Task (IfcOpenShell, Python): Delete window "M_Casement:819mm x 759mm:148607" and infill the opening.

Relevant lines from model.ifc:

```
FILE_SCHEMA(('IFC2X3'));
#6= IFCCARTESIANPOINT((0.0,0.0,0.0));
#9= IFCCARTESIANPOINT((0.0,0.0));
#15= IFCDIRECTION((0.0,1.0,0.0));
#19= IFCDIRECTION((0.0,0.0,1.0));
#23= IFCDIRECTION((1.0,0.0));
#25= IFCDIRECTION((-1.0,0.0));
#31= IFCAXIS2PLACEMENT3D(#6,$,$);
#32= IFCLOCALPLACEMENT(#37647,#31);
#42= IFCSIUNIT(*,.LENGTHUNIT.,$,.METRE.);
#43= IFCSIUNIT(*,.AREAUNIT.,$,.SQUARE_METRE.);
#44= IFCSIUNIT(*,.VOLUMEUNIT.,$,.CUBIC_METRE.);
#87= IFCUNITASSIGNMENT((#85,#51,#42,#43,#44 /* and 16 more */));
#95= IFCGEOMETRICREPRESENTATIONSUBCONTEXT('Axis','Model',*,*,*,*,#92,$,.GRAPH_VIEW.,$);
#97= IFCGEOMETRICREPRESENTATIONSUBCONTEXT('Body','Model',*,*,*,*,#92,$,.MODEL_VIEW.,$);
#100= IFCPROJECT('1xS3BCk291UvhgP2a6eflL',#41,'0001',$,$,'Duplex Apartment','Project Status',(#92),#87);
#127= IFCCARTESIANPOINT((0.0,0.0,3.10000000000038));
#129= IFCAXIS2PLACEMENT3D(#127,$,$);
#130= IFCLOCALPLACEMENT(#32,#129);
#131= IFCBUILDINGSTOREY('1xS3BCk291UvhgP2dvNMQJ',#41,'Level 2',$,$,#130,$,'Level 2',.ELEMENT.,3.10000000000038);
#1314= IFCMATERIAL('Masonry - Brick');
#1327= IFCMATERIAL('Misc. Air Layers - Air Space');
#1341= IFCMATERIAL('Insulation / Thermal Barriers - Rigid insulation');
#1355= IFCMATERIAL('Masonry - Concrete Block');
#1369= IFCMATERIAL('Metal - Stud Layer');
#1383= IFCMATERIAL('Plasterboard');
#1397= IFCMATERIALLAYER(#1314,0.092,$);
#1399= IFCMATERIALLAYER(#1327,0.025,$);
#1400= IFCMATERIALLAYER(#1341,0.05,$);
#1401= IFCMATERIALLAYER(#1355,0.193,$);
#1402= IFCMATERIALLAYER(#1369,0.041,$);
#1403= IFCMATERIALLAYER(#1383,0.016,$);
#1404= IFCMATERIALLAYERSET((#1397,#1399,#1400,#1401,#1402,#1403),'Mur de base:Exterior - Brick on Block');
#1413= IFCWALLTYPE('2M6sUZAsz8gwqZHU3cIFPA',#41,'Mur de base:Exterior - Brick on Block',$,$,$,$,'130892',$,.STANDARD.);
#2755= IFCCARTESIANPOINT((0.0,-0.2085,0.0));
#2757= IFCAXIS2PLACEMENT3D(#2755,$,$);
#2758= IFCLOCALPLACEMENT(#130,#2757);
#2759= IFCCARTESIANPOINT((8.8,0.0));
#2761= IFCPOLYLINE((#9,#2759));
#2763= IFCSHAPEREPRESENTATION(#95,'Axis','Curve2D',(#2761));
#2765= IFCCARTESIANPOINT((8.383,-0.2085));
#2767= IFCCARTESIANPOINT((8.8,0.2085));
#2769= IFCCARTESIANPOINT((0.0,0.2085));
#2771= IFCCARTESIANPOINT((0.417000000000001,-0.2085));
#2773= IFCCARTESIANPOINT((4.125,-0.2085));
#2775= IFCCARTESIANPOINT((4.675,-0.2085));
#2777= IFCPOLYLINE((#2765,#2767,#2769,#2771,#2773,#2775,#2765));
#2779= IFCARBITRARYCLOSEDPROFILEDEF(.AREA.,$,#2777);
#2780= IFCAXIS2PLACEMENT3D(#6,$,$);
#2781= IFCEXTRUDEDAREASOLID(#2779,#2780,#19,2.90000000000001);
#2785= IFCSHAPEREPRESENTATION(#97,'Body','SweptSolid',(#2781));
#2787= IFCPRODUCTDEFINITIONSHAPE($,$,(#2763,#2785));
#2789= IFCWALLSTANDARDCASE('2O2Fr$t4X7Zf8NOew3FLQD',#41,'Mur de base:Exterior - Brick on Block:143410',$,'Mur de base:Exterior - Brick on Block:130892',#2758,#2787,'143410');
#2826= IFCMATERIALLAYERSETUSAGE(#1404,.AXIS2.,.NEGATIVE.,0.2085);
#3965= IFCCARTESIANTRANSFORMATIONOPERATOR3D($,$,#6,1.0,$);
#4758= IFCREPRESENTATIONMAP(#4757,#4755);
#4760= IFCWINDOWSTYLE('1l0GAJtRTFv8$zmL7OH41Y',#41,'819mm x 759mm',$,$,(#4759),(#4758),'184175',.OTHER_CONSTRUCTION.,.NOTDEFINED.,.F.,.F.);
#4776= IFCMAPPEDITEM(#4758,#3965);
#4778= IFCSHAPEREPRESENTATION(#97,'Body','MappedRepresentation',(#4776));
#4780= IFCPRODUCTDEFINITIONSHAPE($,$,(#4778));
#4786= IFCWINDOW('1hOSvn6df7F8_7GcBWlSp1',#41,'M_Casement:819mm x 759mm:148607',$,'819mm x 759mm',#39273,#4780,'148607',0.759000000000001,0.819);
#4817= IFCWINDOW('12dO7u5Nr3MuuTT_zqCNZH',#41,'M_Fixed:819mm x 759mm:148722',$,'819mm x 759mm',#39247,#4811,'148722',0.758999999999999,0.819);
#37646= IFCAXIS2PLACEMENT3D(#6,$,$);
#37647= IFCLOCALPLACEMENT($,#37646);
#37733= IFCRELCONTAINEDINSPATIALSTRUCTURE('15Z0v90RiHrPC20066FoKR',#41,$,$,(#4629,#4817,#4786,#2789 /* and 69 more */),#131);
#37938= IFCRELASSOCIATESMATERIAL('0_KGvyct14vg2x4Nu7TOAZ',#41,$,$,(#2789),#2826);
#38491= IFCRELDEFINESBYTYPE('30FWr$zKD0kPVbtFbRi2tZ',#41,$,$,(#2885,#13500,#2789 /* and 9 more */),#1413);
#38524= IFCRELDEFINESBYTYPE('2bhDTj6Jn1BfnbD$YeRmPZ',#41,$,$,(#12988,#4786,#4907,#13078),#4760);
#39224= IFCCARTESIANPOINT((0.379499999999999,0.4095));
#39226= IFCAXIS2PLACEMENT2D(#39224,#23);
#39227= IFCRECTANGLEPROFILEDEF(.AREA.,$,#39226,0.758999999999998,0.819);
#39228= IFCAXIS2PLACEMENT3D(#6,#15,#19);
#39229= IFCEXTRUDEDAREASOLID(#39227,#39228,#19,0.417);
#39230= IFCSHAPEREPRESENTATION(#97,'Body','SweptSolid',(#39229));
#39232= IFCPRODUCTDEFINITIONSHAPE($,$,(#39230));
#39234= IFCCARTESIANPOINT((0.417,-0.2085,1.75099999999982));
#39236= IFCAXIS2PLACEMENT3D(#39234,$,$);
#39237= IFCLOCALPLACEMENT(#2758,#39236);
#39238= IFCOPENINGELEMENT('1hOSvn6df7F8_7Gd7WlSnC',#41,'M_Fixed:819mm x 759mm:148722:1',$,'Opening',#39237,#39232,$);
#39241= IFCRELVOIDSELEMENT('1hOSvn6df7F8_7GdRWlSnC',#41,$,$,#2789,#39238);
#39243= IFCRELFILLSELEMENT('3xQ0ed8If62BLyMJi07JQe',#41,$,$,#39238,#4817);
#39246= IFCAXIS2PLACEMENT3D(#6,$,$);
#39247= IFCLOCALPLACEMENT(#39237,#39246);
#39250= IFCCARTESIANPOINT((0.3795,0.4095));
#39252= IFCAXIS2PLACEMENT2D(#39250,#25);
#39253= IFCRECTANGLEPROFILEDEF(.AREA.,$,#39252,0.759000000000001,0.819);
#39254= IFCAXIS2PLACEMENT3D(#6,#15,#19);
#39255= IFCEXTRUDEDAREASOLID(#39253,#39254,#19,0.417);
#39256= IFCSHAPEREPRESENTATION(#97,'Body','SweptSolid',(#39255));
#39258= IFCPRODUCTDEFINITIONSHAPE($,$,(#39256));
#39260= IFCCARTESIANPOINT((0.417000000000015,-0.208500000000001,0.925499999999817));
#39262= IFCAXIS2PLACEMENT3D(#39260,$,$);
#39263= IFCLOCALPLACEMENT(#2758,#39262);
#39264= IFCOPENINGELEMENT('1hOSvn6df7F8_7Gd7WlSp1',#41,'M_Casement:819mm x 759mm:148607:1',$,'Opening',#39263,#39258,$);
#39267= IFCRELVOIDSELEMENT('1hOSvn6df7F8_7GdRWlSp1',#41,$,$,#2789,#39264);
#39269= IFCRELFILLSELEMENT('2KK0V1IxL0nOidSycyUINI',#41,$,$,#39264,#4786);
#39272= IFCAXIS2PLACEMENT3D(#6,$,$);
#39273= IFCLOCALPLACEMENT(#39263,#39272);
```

```python
import ifcopenshell
import ifcopenshell.api.feature
import ifcopenshell.api.root
import ifcopenshell.geom
import ifcopenshell.util.shape

model = ifcopenshell.open("model.ifc")
settings = ifcopenshell.geom.settings()


def volume(element):
    """Net volume in cubic metres, openings subtracted."""
    shape = ifcopenshell.geom.create_shape(settings, element)
    return ifcopenshell.util.shape.get_volume(shape.geometry)


window = model.by_id(4786)
opening = window.FillsVoids[0].RelatingOpeningElement
wall = opening.VoidsElements[0].RelatingBuildingElement
before = volume(wall)

ifcopenshell.api.root.remove_product(model, product=window)
ifcopenshell.api.feature.remove_feature(model, feature=opening)

after = volume(wall)

print(f"wall volume {before:.3f} -> {after:.3f} m3")

model.write("model_v2.ifc")
```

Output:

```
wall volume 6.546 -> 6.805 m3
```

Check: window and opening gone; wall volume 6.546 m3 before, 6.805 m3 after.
